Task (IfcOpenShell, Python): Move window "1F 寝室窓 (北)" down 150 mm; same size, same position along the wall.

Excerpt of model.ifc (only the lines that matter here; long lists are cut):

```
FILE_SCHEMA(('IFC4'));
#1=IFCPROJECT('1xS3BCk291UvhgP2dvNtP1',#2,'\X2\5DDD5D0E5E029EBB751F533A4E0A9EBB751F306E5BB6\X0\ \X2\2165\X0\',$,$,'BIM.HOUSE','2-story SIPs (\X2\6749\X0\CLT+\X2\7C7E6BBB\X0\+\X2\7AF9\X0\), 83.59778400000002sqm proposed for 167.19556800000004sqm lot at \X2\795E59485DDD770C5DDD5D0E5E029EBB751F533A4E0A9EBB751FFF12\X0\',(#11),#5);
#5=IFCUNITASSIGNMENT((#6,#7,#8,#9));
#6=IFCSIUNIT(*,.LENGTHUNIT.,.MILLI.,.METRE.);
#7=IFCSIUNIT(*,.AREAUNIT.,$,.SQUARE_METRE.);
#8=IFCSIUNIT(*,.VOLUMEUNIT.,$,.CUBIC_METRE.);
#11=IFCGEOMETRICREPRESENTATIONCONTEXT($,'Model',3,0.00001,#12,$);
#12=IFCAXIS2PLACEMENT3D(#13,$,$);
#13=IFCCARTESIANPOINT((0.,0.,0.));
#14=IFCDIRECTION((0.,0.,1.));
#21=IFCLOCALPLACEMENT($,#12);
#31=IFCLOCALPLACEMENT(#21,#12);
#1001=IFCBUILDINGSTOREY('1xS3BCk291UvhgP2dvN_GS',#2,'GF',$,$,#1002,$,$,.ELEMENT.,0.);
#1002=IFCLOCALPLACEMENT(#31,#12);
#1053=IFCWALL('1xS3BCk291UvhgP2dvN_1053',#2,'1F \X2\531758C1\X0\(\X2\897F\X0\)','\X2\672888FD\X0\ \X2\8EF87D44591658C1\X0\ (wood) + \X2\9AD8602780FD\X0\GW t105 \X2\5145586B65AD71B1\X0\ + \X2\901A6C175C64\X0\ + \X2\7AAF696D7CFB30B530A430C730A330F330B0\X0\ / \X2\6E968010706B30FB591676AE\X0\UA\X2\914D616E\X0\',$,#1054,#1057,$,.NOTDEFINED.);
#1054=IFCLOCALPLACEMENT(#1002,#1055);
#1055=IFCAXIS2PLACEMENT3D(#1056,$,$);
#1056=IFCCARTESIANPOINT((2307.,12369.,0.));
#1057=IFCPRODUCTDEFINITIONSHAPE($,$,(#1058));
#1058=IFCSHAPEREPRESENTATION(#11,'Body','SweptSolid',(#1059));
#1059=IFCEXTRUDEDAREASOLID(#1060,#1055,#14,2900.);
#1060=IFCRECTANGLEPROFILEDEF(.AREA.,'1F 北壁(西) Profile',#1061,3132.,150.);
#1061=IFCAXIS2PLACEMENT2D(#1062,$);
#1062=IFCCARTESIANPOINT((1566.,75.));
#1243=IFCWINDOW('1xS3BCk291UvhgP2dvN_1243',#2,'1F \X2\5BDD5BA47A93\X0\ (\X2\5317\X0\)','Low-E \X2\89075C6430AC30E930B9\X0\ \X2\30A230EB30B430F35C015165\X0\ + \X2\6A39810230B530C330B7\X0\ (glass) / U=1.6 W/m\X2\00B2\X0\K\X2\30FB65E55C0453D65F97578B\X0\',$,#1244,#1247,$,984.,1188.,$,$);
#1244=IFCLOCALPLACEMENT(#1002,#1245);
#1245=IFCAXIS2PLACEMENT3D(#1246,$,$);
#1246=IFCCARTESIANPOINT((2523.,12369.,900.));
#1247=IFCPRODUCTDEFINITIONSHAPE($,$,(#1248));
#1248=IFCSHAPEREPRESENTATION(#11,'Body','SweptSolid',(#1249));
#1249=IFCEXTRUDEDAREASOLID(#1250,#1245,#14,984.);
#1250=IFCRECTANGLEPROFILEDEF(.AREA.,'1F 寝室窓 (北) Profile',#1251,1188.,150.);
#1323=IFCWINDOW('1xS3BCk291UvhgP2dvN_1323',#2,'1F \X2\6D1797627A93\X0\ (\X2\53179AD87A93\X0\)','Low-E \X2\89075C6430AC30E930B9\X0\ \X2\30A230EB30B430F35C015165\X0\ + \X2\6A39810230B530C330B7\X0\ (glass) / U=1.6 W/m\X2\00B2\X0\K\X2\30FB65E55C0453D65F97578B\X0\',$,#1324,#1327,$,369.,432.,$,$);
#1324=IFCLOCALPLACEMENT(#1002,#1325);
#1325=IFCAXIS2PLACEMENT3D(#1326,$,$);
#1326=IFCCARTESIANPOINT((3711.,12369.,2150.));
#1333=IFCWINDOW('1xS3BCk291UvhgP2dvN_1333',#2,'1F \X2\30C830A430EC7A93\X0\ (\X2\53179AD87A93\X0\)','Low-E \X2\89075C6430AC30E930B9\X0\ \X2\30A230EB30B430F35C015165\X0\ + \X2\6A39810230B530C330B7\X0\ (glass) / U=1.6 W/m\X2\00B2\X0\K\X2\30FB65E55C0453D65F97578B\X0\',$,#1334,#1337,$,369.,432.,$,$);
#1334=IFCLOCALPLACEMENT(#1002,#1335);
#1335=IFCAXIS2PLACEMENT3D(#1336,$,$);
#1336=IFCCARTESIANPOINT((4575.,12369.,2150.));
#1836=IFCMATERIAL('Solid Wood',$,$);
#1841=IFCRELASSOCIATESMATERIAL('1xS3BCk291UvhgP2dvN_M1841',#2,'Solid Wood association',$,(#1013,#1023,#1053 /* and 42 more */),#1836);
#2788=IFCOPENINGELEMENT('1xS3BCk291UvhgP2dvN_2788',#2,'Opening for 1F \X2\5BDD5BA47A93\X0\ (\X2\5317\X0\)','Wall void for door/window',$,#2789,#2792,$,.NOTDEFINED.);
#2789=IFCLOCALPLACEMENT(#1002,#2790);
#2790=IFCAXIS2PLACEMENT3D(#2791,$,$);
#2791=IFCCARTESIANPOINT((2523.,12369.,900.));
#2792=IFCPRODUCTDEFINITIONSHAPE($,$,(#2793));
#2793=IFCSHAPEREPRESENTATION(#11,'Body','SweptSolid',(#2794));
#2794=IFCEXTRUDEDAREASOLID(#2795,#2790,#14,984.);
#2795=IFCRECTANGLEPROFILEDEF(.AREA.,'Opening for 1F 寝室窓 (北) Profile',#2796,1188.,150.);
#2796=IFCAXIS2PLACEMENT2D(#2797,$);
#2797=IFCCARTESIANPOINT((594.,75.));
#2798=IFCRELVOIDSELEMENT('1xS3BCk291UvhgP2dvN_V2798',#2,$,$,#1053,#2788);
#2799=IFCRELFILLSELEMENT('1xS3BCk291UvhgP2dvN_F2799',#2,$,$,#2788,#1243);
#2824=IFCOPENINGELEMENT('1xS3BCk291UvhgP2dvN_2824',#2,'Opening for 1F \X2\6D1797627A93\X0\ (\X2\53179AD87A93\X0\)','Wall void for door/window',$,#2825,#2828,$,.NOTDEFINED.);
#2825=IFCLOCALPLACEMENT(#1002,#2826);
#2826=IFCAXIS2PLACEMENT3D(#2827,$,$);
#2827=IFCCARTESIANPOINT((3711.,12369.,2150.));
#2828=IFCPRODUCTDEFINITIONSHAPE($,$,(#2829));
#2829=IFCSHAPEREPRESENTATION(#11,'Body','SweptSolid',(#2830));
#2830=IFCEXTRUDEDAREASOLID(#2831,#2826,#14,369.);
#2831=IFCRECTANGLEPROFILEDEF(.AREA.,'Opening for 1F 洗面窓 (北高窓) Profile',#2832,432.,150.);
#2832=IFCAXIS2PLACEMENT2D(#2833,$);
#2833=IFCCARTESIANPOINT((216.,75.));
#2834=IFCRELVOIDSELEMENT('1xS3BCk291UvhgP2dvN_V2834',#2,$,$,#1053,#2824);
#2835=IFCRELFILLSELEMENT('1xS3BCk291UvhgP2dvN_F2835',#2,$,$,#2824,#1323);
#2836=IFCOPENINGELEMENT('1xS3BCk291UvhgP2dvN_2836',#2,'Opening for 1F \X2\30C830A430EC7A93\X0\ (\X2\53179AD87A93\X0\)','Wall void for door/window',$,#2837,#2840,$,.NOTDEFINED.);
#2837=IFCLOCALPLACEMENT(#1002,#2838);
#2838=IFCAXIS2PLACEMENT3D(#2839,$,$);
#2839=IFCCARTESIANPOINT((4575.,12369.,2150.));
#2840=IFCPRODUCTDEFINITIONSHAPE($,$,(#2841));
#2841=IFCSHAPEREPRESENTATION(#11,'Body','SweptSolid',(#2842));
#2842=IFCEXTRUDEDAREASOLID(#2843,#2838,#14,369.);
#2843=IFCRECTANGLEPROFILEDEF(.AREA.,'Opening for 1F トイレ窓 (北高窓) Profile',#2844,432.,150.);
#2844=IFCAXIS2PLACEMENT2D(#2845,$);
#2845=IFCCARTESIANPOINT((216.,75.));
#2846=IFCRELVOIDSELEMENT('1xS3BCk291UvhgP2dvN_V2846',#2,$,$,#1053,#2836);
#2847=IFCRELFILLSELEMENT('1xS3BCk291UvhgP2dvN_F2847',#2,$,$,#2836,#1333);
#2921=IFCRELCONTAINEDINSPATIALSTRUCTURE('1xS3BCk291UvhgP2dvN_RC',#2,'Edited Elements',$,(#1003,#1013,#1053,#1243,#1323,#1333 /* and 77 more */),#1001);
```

```python
import numpy as np
import ifcopenshell
import ifcopenshell.api.geometry
import ifcopenshell.util.placement
import ifcopenshell.util.unit

model = ifcopenshell.open("model.ifc")
unit_scale = ifcopenshell.util.unit.calculate_unit_scale(model)

window = model.by_id(1243)
opening = window.FillsVoids[0].RelatingOpeningElement
dz = -150.0

shift = np.array([0.0, 0.0, dz])
# The window is not placed relative to its opening, so move both.
for product in (opening, window):
    matrix = ifcopenshell.util.placement.get_local_placement(product.ObjectPlacement)
    matrix[:3, 3] += shift
    ifcopenshell.api.geometry.edit_object_placement(model, product=product, matrix=matrix, is_si=False)

print(f"moved by {dz * unit_scale:+.3f} m")

model.write("model_edited.ifc")
```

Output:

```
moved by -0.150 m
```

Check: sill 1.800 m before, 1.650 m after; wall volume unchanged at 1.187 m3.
